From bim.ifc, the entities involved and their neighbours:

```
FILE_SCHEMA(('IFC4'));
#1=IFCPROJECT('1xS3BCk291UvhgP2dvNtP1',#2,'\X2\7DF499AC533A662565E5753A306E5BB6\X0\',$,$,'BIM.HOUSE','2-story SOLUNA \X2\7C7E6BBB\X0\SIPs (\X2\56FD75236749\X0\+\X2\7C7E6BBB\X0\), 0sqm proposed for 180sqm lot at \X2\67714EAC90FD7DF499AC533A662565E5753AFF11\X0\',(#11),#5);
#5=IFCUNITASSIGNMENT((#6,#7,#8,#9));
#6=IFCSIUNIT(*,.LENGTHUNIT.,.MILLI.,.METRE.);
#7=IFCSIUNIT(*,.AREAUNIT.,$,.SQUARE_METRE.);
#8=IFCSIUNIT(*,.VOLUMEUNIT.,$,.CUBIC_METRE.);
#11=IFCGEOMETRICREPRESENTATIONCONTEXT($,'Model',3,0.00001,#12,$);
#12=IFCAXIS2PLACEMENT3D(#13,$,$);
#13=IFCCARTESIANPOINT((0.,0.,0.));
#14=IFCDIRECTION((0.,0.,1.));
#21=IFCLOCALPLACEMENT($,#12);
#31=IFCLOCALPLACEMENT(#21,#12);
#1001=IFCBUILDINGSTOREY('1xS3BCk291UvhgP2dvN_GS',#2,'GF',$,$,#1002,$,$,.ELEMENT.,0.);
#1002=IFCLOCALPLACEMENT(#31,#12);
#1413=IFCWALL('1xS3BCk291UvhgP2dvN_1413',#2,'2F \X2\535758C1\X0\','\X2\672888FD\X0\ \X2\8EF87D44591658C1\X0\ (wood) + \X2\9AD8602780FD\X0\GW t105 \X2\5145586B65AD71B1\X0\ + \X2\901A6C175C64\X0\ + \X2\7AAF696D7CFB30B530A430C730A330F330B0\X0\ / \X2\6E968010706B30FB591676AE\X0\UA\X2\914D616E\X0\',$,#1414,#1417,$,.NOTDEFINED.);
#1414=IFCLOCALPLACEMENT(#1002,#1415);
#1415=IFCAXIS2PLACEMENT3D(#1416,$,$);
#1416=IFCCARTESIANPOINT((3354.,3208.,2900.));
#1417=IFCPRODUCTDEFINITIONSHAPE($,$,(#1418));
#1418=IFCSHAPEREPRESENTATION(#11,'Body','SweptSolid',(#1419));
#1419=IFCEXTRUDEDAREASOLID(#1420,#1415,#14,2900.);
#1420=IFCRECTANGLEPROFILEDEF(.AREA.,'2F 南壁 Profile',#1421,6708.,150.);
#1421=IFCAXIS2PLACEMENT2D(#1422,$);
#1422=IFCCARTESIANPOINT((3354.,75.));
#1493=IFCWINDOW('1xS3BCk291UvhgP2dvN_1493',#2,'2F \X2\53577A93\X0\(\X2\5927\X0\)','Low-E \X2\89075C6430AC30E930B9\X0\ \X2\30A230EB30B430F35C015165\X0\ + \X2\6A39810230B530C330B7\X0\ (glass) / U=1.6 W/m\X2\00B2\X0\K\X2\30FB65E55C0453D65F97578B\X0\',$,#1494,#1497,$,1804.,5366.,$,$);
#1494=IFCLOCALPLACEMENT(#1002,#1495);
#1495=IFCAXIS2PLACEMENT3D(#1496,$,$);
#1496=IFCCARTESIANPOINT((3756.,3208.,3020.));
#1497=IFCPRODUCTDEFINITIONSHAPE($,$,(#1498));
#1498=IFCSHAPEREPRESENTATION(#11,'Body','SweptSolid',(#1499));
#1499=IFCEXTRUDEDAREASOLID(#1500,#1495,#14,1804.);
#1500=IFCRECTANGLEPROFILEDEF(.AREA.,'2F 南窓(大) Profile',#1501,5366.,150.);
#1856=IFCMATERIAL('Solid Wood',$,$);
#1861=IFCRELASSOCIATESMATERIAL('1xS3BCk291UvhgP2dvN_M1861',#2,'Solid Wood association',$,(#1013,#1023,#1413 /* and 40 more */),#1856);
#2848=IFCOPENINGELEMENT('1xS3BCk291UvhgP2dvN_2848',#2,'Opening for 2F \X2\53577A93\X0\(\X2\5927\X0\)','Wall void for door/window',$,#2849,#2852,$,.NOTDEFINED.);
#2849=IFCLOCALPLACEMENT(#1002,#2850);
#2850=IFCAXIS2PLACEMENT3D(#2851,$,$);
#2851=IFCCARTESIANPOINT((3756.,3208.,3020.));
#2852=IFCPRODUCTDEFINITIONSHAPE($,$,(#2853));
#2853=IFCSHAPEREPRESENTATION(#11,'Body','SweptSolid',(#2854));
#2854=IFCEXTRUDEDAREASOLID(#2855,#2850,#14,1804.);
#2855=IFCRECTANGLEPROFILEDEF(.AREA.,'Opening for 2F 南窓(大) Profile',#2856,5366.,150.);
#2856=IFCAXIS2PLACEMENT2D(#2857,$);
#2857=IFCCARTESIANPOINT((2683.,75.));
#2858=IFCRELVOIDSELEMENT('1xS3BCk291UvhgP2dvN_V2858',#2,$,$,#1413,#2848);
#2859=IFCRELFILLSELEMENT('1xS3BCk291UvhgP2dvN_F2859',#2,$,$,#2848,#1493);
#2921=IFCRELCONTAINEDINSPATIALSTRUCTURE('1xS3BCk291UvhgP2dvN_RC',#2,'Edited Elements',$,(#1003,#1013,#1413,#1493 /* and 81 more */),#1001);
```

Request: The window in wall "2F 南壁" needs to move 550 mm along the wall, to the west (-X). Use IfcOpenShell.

```python
import ifcopenshell
import ifcopenshell.api.geometry
import ifcopenshell.util.placement
import ifcopenshell.util.unit

model = ifcopenshell.open("bim.ifc")
unit_scale = ifcopenshell.util.unit.calculate_unit_scale(model)

window = model.by_id(1493)
opening = window.FillsVoids[0].RelatingOpeningElement
wall = opening.VoidsElements[0].RelatingBuildingElement

wall_matrix = ifcopenshell.util.placement.get_local_placement(wall.ObjectPlacement)
shift = wall_matrix[:3, 0] * -0.55 / unit_scale
before = ifcopenshell.util.placement.get_local_placement(window.ObjectPlacement)[:3, 3].copy()

# The window is not placed relative to its opening, so move both.
for product in (opening, window):
    matrix = ifcopenshell.util.placement.get_local_placement(product.ObjectPlacement)
    matrix[:3, 3] += shift
    ifcopenshell.api.geometry.edit_object_placement(model, product=product, matrix=matrix, is_si=False)

after = ifcopenshell.util.placement.get_local_placement(window.ObjectPlacement)[:3, 3]
print("window moved by", (after - before).round(3) + 0.0)

model.write("bim_edited.ifc")
```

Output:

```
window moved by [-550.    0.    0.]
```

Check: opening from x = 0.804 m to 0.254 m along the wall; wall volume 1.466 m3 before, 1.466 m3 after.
